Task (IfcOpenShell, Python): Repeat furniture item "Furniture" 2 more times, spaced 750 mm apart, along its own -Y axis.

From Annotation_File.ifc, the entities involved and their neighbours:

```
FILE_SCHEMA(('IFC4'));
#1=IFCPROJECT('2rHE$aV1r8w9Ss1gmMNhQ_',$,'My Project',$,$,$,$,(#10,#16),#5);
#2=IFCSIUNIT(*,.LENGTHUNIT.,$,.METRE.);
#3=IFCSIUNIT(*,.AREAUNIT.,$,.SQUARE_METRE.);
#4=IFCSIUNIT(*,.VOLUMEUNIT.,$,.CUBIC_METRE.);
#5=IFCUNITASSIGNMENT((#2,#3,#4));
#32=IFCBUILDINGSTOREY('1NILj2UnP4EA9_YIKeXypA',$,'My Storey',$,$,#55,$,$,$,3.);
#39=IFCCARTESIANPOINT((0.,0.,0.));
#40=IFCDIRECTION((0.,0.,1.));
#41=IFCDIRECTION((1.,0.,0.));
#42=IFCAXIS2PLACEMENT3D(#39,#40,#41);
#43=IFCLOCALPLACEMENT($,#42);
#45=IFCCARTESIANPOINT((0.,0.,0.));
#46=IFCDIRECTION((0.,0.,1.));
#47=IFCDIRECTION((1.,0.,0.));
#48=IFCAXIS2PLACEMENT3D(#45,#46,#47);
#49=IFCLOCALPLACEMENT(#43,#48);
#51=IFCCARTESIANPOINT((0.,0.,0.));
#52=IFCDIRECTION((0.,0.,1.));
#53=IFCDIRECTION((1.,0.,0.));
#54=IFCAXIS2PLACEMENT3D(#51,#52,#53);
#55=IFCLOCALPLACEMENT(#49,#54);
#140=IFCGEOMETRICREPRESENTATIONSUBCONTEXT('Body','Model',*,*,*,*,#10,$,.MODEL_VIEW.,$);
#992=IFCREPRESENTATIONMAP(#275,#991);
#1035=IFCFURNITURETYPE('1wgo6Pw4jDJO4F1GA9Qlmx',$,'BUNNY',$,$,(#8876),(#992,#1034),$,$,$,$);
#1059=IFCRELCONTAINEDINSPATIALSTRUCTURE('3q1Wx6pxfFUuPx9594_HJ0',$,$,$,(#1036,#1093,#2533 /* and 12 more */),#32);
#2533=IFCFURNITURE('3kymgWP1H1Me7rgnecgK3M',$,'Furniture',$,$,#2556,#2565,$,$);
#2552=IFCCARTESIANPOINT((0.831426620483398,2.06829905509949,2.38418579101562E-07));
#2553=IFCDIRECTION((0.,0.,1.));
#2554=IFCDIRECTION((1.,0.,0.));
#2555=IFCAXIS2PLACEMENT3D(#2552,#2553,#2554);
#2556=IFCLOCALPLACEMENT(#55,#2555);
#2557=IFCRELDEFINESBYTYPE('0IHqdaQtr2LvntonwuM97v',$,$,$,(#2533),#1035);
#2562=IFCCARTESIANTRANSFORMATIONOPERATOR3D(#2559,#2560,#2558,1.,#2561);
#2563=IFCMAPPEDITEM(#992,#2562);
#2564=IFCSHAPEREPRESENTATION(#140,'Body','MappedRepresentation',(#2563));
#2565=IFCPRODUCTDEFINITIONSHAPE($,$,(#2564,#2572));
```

```python
import ifcopenshell
import ifcopenshell.api.geometry
import ifcopenshell.api.root
import ifcopenshell.util.element
import ifcopenshell.util.placement
import ifcopenshell.util.unit

model = ifcopenshell.open("Annotation_File.ifc")
unit_scale = ifcopenshell.util.unit.calculate_unit_scale(model)

source = model.by_guid("3kymgWP1H1Me7rgnecgK3M")
base = ifcopenshell.util.placement.get_local_placement(source.ObjectPlacement)
step = -base[:3, 1] * 0.75 / unit_scale

for i in range(1, 3):
    copy = ifcopenshell.api.root.copy_class(model, product=source)
    copy.Representation = ifcopenshell.util.element.copy_deep(
        model, source.Representation, exclude=["IfcGeometricRepresentationContext", "IfcRepresentationMap"]
    )
    matrix = base.copy()
    matrix[:3, 3] += i * step
    print("added at", matrix[:3, 3].round(3) + 0.0)
    ifcopenshell.api.geometry.edit_object_placement(model, product=copy, matrix=matrix, is_si=False)

model.write("Annotation_File_edited.ifc")
```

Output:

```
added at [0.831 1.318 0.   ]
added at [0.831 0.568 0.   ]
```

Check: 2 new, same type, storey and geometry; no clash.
